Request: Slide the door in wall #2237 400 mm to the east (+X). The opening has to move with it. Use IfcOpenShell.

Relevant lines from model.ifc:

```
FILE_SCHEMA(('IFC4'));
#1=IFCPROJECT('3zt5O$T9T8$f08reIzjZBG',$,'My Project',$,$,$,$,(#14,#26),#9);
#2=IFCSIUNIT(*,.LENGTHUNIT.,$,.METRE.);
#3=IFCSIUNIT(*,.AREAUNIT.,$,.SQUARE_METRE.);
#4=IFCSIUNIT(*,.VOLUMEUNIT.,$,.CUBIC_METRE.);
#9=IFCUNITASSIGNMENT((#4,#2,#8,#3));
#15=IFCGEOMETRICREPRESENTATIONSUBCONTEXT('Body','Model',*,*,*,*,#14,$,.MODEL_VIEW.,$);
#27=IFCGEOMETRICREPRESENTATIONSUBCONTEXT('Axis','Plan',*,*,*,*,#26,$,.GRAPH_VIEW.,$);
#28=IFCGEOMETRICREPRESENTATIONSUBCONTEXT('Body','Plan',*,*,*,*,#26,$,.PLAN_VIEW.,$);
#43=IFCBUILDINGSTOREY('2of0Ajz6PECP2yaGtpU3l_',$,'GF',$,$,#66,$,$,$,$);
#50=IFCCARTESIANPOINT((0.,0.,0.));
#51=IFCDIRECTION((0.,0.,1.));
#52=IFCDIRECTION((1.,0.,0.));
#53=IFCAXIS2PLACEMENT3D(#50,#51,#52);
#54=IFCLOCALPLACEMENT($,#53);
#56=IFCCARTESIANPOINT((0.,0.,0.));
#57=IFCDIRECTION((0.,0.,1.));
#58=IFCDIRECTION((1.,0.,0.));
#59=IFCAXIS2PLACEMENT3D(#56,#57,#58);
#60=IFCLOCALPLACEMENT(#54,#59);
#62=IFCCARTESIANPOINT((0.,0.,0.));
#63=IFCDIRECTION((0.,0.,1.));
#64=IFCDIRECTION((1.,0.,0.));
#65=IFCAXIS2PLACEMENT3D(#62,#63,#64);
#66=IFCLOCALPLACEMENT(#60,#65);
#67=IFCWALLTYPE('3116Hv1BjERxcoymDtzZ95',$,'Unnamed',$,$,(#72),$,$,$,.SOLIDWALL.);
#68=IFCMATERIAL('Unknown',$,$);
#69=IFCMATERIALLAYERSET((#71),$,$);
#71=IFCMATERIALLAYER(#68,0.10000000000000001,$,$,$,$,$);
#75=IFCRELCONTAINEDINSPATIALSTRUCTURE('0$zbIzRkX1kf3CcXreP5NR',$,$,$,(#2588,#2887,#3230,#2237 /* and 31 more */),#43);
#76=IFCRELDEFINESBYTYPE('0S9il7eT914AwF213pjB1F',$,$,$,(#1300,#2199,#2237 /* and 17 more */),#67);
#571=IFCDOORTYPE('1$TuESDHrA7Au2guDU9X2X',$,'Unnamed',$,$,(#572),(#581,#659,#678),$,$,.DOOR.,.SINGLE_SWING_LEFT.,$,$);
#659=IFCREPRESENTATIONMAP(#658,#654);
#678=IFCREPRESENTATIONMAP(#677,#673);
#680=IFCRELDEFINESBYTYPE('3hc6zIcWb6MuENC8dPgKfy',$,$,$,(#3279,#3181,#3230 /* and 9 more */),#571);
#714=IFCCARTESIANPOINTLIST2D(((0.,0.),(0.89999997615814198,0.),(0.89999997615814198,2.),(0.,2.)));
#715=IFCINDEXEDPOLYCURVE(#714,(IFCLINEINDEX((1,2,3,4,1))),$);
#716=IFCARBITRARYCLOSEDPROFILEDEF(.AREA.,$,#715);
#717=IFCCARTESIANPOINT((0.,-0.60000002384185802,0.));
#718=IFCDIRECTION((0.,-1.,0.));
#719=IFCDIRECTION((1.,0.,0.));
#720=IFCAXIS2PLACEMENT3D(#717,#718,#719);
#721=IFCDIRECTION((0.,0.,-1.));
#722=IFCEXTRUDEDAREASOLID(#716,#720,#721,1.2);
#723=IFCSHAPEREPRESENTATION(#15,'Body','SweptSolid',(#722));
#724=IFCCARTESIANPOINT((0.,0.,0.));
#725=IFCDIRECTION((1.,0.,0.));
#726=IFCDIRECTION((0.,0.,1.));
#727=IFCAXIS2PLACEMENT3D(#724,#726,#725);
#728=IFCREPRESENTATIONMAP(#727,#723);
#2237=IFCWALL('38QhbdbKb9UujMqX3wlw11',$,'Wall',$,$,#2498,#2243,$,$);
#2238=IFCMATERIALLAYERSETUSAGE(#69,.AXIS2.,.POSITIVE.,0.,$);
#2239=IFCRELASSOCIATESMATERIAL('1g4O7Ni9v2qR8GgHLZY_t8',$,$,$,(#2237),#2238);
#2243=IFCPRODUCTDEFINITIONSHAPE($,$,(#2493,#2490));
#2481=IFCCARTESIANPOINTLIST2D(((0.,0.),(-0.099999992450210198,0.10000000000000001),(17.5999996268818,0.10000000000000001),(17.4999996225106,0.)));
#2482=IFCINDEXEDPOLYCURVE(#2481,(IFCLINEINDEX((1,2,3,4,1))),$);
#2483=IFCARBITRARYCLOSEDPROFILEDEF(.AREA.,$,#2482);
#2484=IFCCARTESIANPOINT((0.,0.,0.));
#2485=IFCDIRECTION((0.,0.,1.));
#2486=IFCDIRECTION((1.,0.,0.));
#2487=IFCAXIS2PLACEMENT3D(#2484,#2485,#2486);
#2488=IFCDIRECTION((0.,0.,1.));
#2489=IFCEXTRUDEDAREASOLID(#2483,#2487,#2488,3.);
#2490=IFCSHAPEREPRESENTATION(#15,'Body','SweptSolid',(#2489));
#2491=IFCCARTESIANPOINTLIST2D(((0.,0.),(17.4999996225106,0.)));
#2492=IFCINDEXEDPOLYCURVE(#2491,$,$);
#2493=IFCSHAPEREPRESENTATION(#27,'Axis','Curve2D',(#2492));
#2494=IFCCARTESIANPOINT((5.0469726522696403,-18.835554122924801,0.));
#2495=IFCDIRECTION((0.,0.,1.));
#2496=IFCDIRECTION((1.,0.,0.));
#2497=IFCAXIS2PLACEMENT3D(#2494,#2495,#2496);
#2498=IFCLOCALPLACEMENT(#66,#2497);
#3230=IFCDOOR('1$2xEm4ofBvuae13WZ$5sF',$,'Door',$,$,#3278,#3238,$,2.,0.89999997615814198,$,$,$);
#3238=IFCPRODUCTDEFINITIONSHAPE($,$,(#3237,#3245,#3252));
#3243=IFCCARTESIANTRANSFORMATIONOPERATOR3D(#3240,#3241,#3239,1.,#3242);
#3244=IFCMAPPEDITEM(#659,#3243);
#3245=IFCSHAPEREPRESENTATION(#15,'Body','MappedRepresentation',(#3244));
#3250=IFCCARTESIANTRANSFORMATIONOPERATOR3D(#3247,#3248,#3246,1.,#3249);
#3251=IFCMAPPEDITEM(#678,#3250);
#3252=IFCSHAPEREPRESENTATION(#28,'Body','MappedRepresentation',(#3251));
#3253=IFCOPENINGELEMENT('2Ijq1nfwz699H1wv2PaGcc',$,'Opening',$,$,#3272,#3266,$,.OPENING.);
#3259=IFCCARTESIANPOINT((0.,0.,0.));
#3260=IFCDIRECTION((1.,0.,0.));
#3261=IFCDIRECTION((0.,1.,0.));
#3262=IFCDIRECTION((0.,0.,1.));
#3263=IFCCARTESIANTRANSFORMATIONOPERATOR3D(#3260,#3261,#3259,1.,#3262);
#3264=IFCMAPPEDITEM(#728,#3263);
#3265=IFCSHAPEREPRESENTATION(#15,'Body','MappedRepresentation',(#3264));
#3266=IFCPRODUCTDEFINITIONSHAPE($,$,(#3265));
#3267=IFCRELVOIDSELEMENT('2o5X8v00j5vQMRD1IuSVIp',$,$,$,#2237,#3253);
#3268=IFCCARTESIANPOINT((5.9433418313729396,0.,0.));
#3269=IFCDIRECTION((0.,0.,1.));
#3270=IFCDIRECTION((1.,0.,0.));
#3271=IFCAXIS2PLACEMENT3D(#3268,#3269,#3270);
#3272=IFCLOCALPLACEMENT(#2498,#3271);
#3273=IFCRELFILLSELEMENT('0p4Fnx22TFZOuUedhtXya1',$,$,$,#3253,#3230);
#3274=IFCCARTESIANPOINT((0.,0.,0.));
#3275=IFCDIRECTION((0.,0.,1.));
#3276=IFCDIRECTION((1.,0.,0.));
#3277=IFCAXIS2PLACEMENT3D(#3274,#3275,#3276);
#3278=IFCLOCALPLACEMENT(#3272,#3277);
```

```python
import ifcopenshell
import ifcopenshell.api.geometry
import ifcopenshell.util.placement
import ifcopenshell.util.unit

model = ifcopenshell.open("model.ifc")
unit_scale = ifcopenshell.util.unit.calculate_unit_scale(model)

door = model.by_guid("1$2xEm4ofBvuae13WZ$5sF")
opening = door.FillsVoids[0].RelatingOpeningElement
wall = opening.VoidsElements[0].RelatingBuildingElement

wall_matrix = ifcopenshell.util.placement.get_local_placement(wall.ObjectPlacement)
shift = wall_matrix[:3, 0] * 0.4 / unit_scale
before = ifcopenshell.util.placement.get_local_placement(door.ObjectPlacement)[:3, 3].copy()

# The door is placed relative to its opening, so it follows when the opening moves.
matrix = ifcopenshell.util.placement.get_local_placement(opening.ObjectPlacement)
matrix[:3, 3] += shift
ifcopenshell.api.geometry.edit_object_placement(
    model, product=opening, matrix=matrix, is_si=False, should_transform_children=True
)

after = ifcopenshell.util.placement.get_local_placement(door.ObjectPlacement)[:3, 3]
print("door moved by", (after - before).round(3) + 0.0)

model.write("model_updated.ifc")
```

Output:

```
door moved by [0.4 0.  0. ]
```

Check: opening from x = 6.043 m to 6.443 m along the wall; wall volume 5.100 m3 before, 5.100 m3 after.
